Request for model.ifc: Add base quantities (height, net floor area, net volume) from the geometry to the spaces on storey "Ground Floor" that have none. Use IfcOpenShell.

First a look at what the model holds.

```python
import ifcopenshell
import ifcopenshell.util.element
import ifcopenshell.util.unit

model = ifcopenshell.open("model.ifc")
print(model.schema)
for unit_type in ("LENGTHUNIT", "AREAUNIT", "VOLUMEUNIT"):
    print(unit_type, ifcopenshell.util.unit.calculate_unit_scale(model, unit_type))
storey = next(s for s in model.by_type("IfcBuildingStorey") if s.Name == "Ground Floor")
spaces = [e for e in ifcopenshell.util.element.get_decomposition(storey) if e.is_a("IfcSpace")]
for e in sorted(spaces, key=lambda e: e.id()):
    print(e.id(), e.is_a(), e.Name, list(ifcopenshell.util.element.get_psets(e, qtos_only=True)), sep=" | ")
```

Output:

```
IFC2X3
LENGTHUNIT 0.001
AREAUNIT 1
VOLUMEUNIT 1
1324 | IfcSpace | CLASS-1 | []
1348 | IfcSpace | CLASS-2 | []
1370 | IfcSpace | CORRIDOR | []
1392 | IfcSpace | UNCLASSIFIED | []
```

```python
import ifcopenshell
import ifcopenshell.api.pset
import ifcopenshell.geom
import ifcopenshell.util.element
import ifcopenshell.util.shape
import ifcopenshell.util.unit

model = ifcopenshell.open("model.ifc")
unit_scale = ifcopenshell.util.unit.calculate_unit_scale(model)
area_scale = ifcopenshell.util.unit.calculate_unit_scale(model, "AREAUNIT")
volume_scale = ifcopenshell.util.unit.calculate_unit_scale(model, "VOLUMEUNIT")
settings = ifcopenshell.geom.settings()

storey = next(s for s in model.by_type("IfcBuildingStorey") if s.Name == "Ground Floor")
spaces = [e for e in ifcopenshell.util.element.get_decomposition(storey) if e.is_a("IfcSpace")]

for e in sorted(spaces, key=lambda e: e.id()):
    if ifcopenshell.util.element.get_psets(e, qtos_only=True, should_inherit=False):
        continue
    # Geometry comes back in metres, in the element's own axes.
    shape = ifcopenshell.geom.create_shape(settings, e)
    values = {
        "Height": ifcopenshell.util.shape.get_z(shape.geometry) / unit_scale,
        "NetFloorArea": ifcopenshell.util.shape.get_footprint_area(shape.geometry) / area_scale,
        "NetVolume": ifcopenshell.util.shape.get_volume(shape.geometry) / volume_scale,
    }
    qto = ifcopenshell.api.pset.add_qto(model, product=e, name="BaseQuantities")
    ifcopenshell.api.pset.edit_qto(model, qto=qto, properties=values)
    print(e.id(), {k: round(v, 3) for k, v in values.items()})

model.write("model_edited.ifc")
```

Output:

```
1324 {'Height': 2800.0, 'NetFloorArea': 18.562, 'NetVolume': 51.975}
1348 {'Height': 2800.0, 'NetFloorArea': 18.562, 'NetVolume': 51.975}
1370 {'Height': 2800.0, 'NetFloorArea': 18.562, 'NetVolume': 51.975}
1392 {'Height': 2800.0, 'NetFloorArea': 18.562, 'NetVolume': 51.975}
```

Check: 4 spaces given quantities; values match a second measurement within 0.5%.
